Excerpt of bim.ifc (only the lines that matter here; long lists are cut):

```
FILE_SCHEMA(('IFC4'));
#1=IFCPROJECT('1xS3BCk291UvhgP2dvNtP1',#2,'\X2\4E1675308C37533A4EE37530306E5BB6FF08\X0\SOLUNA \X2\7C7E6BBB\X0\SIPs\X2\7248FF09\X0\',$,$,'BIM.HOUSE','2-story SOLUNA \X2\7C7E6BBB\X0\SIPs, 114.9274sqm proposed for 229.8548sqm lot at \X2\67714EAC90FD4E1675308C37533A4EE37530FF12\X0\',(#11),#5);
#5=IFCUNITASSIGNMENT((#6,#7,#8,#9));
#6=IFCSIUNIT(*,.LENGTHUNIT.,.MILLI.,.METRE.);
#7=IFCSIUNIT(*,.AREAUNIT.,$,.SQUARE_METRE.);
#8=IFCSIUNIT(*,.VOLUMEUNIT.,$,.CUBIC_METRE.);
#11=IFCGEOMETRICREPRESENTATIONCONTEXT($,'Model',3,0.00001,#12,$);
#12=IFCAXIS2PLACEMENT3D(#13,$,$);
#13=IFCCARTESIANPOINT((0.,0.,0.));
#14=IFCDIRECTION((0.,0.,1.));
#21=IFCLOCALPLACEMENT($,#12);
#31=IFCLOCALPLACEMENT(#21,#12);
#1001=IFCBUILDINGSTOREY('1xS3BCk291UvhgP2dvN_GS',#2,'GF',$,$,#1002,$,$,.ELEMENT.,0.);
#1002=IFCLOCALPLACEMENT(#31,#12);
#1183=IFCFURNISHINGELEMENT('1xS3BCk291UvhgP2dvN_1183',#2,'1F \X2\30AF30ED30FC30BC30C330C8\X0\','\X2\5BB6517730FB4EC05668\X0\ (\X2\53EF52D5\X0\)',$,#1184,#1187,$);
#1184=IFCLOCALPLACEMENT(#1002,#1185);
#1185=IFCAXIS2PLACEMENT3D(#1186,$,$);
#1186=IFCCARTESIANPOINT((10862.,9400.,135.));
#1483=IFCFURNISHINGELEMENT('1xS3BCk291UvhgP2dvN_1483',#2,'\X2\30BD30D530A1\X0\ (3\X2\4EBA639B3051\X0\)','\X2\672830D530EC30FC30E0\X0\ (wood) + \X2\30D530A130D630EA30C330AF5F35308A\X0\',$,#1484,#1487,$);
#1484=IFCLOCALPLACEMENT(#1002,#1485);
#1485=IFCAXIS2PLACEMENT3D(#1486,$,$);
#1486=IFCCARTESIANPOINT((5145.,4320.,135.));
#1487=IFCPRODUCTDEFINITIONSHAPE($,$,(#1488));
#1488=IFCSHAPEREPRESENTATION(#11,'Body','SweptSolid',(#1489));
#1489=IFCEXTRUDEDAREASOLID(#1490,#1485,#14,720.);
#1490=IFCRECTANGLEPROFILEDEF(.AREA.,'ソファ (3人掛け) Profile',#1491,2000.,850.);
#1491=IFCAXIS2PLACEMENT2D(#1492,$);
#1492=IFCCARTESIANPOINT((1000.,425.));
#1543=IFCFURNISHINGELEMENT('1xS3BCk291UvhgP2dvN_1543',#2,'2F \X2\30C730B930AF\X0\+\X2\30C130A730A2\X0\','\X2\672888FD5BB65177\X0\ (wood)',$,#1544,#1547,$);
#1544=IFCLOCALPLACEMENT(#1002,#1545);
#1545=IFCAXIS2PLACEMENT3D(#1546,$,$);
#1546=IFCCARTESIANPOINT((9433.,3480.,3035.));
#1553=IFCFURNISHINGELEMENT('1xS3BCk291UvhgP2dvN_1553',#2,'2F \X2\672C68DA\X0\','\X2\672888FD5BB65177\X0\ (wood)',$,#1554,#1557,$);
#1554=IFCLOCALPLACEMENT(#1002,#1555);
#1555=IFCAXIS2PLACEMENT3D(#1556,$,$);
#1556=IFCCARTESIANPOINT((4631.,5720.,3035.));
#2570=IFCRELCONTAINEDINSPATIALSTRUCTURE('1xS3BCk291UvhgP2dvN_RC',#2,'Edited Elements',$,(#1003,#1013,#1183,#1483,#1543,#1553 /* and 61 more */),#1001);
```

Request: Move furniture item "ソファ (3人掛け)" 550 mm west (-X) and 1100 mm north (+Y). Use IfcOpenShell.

```python
import ifcopenshell
import ifcopenshell.api.geometry
import ifcopenshell.util.placement

model = ifcopenshell.open("bim.ifc")

item = model.by_guid("1xS3BCk291UvhgP2dvN_1483")
matrix = ifcopenshell.util.placement.get_local_placement(item.ObjectPlacement)
matrix[0, 3] -= 550.0
matrix[1, 3] += 1100.0
ifcopenshell.api.geometry.edit_object_placement(model, product=item, matrix=matrix, is_si=False)

print(ifcopenshell.util.placement.get_local_placement(item.ObjectPlacement).round(3) + 0.0)

model.write("bim_edited.ifc")
```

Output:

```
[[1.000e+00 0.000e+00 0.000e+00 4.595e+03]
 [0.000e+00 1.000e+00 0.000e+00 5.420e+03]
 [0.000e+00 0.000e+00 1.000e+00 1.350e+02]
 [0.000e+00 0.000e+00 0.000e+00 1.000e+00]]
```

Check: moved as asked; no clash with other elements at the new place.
